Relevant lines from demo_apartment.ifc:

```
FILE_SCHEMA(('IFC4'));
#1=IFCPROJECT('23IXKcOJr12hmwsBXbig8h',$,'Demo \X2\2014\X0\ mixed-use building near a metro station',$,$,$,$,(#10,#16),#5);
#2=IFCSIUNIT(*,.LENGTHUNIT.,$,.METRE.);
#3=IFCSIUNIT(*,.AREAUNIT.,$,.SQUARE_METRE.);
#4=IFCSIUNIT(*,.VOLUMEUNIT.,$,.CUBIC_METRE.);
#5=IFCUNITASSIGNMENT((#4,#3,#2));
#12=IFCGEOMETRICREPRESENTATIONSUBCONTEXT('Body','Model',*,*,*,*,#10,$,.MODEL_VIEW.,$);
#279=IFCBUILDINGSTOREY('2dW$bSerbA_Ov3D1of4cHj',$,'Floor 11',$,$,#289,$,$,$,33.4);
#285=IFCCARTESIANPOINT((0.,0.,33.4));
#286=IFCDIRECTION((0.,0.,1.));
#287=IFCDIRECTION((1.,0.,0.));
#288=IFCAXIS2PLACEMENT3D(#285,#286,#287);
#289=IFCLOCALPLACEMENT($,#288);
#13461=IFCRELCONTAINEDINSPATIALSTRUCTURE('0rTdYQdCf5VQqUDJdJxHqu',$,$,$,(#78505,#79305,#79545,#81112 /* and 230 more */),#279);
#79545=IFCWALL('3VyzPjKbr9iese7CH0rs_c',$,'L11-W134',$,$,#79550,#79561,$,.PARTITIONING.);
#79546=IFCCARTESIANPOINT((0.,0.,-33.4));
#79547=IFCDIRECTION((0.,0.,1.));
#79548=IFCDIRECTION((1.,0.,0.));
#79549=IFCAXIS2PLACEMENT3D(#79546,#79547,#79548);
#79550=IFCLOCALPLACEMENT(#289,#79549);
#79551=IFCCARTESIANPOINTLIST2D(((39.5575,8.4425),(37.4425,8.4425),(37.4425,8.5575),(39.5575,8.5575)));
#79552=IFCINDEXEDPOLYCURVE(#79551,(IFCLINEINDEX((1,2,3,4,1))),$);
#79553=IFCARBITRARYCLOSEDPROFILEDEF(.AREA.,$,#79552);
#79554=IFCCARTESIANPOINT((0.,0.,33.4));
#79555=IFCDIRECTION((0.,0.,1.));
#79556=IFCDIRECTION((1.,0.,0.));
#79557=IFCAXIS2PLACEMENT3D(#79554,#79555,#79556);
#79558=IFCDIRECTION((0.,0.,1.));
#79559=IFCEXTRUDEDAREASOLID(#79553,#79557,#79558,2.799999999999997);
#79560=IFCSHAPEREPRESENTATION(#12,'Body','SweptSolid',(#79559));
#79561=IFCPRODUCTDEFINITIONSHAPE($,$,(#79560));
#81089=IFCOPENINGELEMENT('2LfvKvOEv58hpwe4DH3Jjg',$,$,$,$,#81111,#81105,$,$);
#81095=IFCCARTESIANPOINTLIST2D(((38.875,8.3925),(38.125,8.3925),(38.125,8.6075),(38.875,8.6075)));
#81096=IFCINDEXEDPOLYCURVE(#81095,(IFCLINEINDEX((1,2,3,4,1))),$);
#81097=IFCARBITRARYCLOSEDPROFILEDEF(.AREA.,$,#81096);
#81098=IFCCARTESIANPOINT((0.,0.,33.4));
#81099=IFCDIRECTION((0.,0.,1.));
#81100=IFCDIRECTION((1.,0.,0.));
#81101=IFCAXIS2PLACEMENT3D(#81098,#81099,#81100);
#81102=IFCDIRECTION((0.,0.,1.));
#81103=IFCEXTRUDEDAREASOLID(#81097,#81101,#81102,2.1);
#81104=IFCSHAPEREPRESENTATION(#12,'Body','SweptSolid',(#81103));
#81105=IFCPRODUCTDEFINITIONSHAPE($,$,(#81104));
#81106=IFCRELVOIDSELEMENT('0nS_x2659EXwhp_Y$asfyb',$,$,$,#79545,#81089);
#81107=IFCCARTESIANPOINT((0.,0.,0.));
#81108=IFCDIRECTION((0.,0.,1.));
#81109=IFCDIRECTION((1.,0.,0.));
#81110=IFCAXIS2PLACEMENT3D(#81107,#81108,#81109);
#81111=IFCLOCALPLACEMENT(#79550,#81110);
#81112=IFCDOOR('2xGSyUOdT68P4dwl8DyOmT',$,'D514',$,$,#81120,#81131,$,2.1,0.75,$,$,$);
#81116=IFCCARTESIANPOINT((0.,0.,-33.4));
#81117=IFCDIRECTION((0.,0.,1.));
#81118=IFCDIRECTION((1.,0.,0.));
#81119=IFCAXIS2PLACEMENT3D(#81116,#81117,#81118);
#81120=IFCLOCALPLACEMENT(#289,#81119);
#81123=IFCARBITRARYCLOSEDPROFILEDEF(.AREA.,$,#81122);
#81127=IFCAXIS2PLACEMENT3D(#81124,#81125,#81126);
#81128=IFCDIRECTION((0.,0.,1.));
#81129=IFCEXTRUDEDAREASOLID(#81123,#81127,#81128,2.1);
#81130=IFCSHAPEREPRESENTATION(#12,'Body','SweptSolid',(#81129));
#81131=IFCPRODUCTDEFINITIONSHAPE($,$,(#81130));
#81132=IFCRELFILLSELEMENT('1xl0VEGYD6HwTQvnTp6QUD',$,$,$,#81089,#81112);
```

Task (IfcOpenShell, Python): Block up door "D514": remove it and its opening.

```python
import ifcopenshell
import ifcopenshell.api.feature
import ifcopenshell.api.root
import ifcopenshell.geom
import ifcopenshell.util.shape

model = ifcopenshell.open("demo_apartment.ifc")
settings = ifcopenshell.geom.settings()


def volume(element):
    """Net volume in cubic metres, openings subtracted."""
    shape = ifcopenshell.geom.create_shape(settings, element)
    return ifcopenshell.util.shape.get_volume(shape.geometry)


door = model.by_id(81112)
opening = door.FillsVoids[0].RelatingOpeningElement
wall = opening.VoidsElements[0].RelatingBuildingElement
before = volume(wall)

ifcopenshell.api.root.remove_product(model, product=door)
ifcopenshell.api.feature.remove_feature(model, feature=opening)

after = volume(wall)

print(f"wall volume {before:.3f} -> {after:.3f} m3")

model.write("demo_apartment_rev.ifc")
```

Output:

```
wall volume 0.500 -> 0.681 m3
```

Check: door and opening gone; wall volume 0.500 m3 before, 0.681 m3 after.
